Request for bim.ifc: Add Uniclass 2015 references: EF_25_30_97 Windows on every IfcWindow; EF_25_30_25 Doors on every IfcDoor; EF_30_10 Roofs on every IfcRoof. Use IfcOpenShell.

First a look at what the model holds.

```python
import ifcopenshell

model = ifcopenshell.open("bim.ifc")
print(model.schema)
print("classifications:", [c.Name for c in model.by_type("IfcClassification")])
for ifc_class in ("IfcDoor", "IfcRoof", "IfcStair", "IfcWall", "IfcWindow"):
    print(ifc_class, len(model.by_type(ifc_class)))
```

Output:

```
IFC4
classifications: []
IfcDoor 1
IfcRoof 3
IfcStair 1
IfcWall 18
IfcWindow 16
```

```python
import ifcopenshell
import ifcopenshell.api.classification

model = ifcopenshell.open("bim.ifc")

system = ifcopenshell.api.classification.add_classification(model, classification="Uniclass 2015")

codes = {
    "IfcWindow": ("EF_25_30_97", "Windows"),
    "IfcDoor": ("EF_25_30_25", "Doors"),
    "IfcRoof": ("EF_30_10", "Roofs"),
}
for ifc_class, (code, name) in codes.items():
    products = model.by_type(ifc_class)
    ifcopenshell.api.classification.add_reference(
        model, products=products, classification=system, identification=code, name=name
    )
    print(code, len(products))

model.write("bim-out.ifc")
```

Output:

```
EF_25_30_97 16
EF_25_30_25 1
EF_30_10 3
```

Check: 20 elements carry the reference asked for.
